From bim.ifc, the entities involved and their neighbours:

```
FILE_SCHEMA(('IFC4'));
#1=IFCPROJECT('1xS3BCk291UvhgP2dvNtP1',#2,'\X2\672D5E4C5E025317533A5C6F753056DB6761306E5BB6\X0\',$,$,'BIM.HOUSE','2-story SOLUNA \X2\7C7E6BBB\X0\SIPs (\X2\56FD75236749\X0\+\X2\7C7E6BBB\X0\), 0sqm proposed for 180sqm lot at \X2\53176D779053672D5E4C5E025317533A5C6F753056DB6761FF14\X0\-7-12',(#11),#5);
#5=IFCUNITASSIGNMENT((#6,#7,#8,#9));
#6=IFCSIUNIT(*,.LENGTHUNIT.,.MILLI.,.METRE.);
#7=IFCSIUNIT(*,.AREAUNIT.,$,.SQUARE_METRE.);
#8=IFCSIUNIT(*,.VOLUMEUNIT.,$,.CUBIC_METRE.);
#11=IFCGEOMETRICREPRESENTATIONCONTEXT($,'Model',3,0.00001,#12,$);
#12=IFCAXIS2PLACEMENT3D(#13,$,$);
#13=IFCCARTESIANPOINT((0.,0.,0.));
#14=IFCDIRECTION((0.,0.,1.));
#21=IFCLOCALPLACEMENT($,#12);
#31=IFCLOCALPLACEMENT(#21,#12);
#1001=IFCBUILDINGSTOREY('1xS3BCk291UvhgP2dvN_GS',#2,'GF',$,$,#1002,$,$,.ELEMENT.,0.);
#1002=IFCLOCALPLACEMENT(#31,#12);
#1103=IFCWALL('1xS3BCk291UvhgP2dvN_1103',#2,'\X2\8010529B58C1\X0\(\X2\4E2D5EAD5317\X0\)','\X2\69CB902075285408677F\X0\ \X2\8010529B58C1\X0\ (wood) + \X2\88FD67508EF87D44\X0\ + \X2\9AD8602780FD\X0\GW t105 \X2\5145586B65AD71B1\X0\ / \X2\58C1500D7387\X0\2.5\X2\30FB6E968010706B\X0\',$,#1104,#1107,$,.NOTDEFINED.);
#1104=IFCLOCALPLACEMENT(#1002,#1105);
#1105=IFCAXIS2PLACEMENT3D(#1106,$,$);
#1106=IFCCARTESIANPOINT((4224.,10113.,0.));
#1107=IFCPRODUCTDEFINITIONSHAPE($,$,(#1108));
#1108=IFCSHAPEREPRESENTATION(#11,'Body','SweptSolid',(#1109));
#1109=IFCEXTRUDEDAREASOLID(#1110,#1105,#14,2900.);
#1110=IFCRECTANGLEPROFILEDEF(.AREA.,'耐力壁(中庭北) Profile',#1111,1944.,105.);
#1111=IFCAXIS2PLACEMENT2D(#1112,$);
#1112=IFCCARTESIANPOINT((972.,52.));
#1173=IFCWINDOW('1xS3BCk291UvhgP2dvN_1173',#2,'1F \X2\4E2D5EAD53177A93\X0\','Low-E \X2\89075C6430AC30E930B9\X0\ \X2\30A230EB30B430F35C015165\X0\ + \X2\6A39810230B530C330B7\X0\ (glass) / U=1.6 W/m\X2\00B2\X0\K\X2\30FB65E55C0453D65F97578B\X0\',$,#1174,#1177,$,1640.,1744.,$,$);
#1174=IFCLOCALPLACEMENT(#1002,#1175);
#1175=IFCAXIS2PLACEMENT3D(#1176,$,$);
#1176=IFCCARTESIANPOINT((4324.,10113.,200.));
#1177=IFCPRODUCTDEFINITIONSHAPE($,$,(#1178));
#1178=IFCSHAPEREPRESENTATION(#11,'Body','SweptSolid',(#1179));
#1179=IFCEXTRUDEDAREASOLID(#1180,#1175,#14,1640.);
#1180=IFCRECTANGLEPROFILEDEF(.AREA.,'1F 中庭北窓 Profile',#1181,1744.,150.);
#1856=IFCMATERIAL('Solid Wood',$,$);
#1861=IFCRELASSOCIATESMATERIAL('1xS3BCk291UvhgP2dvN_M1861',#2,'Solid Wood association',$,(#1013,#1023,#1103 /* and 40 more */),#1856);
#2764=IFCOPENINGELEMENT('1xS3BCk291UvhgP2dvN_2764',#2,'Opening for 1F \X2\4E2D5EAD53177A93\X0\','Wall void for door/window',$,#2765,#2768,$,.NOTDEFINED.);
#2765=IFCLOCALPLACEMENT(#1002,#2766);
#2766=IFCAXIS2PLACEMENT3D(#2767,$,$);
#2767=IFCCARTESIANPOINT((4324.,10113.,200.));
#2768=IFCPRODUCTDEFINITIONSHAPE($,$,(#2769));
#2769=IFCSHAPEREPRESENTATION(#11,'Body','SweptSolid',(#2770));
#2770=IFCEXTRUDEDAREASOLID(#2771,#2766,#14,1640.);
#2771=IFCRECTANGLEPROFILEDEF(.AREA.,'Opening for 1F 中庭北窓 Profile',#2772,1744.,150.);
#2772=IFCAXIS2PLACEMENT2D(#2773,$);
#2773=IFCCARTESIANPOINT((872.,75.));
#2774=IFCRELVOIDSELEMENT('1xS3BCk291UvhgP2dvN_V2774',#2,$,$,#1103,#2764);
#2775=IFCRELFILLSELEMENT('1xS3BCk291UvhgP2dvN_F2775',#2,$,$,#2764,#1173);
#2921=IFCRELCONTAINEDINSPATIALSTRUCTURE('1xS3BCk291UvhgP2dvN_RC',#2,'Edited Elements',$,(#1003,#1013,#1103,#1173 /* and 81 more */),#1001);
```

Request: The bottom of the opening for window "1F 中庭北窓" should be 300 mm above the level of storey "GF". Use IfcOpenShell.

```python
import numpy as np
import ifcopenshell
import ifcopenshell.api.geometry
import ifcopenshell.geom
import ifcopenshell.util.element
import ifcopenshell.util.placement
import ifcopenshell.util.shape
import ifcopenshell.util.unit

model = ifcopenshell.open("bim.ifc")
unit_scale = ifcopenshell.util.unit.calculate_unit_scale(model)

window = model.by_guid("1xS3BCk291UvhgP2dvN_1173")
opening = window.FillsVoids[0].RelatingOpeningElement
storey = ifcopenshell.util.element.get_container(window, ifc_class="IfcBuildingStorey")
level = ifcopenshell.util.placement.get_local_placement(storey.ObjectPlacement)[2, 3]

# The opening's origin need not be at the sill, so measure its lowest point.
shape = ifcopenshell.geom.create_shape(ifcopenshell.geom.settings(), opening)
bottom = ifcopenshell.util.shape.get_shape_bottom_elevation(shape, shape.geometry) / unit_scale
dz = level + 300.0 - bottom

shift = np.array([0.0, 0.0, dz])
# The window is not placed relative to its opening, so move both.
for product in (opening, window):
    matrix = ifcopenshell.util.placement.get_local_placement(product.ObjectPlacement)
    matrix[:3, 3] += shift
    ifcopenshell.api.geometry.edit_object_placement(model, product=product, matrix=matrix, is_si=False)

print(f"moved by {dz * unit_scale:+.3f} m")

model.write("bim_edited.ifc")
```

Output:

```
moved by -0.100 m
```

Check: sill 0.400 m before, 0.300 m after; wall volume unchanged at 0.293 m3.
